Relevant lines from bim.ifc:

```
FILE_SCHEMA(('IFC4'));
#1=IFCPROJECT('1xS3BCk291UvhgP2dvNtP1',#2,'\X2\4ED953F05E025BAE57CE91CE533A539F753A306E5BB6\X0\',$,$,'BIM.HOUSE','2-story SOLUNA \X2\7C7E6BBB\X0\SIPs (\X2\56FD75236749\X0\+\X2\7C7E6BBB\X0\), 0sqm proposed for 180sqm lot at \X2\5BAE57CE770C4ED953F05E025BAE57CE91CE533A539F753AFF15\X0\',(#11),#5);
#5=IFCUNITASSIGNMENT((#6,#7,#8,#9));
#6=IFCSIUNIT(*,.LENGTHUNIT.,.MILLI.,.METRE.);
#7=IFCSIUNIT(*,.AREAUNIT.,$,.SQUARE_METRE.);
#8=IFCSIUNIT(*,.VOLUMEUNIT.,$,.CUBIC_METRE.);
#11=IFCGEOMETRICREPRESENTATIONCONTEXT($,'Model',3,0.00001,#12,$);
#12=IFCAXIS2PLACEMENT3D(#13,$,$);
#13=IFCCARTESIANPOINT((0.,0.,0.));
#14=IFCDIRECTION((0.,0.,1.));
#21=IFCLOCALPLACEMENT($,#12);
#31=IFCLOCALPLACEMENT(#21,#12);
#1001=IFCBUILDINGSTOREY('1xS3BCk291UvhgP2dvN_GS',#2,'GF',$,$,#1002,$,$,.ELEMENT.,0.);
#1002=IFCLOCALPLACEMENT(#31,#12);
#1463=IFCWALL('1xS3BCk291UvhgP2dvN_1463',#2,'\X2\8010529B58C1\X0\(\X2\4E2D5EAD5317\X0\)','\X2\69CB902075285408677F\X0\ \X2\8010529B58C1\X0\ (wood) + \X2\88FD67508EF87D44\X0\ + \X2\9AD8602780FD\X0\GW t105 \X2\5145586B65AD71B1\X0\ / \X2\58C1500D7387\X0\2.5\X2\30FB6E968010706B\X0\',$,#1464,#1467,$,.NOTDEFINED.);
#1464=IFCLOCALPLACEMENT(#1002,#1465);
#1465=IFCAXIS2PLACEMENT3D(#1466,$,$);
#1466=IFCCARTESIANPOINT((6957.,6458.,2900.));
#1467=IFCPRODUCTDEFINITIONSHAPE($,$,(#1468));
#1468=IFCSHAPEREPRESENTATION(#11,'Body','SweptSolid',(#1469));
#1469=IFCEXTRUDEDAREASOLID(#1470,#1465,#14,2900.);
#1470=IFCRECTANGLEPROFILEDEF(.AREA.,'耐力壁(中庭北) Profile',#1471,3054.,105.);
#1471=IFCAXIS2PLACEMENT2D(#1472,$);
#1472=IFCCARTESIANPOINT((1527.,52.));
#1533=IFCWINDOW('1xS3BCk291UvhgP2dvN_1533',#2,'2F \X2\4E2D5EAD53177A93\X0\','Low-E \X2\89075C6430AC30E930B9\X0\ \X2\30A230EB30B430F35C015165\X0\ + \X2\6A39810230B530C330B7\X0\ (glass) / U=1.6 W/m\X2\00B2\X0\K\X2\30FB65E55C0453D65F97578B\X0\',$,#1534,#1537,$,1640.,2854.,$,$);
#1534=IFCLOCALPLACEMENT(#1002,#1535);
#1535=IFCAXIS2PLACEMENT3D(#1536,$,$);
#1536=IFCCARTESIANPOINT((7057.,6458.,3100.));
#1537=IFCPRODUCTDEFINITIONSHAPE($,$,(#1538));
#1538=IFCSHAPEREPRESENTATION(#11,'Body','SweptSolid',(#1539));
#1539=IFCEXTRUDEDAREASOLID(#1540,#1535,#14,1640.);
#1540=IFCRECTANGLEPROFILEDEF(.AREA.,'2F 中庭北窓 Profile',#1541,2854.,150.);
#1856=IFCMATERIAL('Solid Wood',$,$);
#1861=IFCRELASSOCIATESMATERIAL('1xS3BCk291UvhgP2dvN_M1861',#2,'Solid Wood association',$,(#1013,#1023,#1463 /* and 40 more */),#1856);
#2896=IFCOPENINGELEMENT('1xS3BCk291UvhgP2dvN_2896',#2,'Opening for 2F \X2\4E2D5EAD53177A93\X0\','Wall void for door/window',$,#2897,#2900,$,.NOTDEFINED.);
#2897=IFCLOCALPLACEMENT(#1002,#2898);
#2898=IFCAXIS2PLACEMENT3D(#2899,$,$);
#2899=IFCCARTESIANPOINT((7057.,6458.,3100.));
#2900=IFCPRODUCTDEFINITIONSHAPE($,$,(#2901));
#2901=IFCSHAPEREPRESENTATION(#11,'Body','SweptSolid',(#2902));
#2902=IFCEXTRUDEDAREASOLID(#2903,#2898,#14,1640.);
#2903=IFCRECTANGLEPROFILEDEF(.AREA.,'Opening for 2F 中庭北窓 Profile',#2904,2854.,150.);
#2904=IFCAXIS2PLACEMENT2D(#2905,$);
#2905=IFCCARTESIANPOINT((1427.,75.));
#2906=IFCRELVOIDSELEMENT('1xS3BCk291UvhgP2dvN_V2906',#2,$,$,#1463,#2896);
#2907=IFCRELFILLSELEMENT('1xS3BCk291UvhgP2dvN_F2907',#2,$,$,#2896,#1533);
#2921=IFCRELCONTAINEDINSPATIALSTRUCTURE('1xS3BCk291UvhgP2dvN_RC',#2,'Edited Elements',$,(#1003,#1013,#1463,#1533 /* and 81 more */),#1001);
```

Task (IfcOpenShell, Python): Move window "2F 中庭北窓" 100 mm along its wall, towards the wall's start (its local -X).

```python
import ifcopenshell
import ifcopenshell.api.geometry
import ifcopenshell.util.placement
import ifcopenshell.util.unit

model = ifcopenshell.open("bim.ifc")
unit_scale = ifcopenshell.util.unit.calculate_unit_scale(model)

window = model.by_id(1533)
opening = window.FillsVoids[0].RelatingOpeningElement
wall = opening.VoidsElements[0].RelatingBuildingElement

wall_matrix = ifcopenshell.util.placement.get_local_placement(wall.ObjectPlacement)
shift = wall_matrix[:3, 0] * -0.1 / unit_scale
before = ifcopenshell.util.placement.get_local_placement(window.ObjectPlacement)[:3, 3].copy()

# The window is not placed relative to its opening, so move both.
for product in (opening, window):
    matrix = ifcopenshell.util.placement.get_local_placement(product.ObjectPlacement)
    matrix[:3, 3] += shift
    ifcopenshell.api.geometry.edit_object_placement(model, product=product, matrix=matrix, is_si=False)

after = ifcopenshell.util.placement.get_local_placement(window.ObjectPlacement)[:3, 3]
print("window moved by", (after - before).round(3) + 0.0)

model.write("bim_edited.ifc")
```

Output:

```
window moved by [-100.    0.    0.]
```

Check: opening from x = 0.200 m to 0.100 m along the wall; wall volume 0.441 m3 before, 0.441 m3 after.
